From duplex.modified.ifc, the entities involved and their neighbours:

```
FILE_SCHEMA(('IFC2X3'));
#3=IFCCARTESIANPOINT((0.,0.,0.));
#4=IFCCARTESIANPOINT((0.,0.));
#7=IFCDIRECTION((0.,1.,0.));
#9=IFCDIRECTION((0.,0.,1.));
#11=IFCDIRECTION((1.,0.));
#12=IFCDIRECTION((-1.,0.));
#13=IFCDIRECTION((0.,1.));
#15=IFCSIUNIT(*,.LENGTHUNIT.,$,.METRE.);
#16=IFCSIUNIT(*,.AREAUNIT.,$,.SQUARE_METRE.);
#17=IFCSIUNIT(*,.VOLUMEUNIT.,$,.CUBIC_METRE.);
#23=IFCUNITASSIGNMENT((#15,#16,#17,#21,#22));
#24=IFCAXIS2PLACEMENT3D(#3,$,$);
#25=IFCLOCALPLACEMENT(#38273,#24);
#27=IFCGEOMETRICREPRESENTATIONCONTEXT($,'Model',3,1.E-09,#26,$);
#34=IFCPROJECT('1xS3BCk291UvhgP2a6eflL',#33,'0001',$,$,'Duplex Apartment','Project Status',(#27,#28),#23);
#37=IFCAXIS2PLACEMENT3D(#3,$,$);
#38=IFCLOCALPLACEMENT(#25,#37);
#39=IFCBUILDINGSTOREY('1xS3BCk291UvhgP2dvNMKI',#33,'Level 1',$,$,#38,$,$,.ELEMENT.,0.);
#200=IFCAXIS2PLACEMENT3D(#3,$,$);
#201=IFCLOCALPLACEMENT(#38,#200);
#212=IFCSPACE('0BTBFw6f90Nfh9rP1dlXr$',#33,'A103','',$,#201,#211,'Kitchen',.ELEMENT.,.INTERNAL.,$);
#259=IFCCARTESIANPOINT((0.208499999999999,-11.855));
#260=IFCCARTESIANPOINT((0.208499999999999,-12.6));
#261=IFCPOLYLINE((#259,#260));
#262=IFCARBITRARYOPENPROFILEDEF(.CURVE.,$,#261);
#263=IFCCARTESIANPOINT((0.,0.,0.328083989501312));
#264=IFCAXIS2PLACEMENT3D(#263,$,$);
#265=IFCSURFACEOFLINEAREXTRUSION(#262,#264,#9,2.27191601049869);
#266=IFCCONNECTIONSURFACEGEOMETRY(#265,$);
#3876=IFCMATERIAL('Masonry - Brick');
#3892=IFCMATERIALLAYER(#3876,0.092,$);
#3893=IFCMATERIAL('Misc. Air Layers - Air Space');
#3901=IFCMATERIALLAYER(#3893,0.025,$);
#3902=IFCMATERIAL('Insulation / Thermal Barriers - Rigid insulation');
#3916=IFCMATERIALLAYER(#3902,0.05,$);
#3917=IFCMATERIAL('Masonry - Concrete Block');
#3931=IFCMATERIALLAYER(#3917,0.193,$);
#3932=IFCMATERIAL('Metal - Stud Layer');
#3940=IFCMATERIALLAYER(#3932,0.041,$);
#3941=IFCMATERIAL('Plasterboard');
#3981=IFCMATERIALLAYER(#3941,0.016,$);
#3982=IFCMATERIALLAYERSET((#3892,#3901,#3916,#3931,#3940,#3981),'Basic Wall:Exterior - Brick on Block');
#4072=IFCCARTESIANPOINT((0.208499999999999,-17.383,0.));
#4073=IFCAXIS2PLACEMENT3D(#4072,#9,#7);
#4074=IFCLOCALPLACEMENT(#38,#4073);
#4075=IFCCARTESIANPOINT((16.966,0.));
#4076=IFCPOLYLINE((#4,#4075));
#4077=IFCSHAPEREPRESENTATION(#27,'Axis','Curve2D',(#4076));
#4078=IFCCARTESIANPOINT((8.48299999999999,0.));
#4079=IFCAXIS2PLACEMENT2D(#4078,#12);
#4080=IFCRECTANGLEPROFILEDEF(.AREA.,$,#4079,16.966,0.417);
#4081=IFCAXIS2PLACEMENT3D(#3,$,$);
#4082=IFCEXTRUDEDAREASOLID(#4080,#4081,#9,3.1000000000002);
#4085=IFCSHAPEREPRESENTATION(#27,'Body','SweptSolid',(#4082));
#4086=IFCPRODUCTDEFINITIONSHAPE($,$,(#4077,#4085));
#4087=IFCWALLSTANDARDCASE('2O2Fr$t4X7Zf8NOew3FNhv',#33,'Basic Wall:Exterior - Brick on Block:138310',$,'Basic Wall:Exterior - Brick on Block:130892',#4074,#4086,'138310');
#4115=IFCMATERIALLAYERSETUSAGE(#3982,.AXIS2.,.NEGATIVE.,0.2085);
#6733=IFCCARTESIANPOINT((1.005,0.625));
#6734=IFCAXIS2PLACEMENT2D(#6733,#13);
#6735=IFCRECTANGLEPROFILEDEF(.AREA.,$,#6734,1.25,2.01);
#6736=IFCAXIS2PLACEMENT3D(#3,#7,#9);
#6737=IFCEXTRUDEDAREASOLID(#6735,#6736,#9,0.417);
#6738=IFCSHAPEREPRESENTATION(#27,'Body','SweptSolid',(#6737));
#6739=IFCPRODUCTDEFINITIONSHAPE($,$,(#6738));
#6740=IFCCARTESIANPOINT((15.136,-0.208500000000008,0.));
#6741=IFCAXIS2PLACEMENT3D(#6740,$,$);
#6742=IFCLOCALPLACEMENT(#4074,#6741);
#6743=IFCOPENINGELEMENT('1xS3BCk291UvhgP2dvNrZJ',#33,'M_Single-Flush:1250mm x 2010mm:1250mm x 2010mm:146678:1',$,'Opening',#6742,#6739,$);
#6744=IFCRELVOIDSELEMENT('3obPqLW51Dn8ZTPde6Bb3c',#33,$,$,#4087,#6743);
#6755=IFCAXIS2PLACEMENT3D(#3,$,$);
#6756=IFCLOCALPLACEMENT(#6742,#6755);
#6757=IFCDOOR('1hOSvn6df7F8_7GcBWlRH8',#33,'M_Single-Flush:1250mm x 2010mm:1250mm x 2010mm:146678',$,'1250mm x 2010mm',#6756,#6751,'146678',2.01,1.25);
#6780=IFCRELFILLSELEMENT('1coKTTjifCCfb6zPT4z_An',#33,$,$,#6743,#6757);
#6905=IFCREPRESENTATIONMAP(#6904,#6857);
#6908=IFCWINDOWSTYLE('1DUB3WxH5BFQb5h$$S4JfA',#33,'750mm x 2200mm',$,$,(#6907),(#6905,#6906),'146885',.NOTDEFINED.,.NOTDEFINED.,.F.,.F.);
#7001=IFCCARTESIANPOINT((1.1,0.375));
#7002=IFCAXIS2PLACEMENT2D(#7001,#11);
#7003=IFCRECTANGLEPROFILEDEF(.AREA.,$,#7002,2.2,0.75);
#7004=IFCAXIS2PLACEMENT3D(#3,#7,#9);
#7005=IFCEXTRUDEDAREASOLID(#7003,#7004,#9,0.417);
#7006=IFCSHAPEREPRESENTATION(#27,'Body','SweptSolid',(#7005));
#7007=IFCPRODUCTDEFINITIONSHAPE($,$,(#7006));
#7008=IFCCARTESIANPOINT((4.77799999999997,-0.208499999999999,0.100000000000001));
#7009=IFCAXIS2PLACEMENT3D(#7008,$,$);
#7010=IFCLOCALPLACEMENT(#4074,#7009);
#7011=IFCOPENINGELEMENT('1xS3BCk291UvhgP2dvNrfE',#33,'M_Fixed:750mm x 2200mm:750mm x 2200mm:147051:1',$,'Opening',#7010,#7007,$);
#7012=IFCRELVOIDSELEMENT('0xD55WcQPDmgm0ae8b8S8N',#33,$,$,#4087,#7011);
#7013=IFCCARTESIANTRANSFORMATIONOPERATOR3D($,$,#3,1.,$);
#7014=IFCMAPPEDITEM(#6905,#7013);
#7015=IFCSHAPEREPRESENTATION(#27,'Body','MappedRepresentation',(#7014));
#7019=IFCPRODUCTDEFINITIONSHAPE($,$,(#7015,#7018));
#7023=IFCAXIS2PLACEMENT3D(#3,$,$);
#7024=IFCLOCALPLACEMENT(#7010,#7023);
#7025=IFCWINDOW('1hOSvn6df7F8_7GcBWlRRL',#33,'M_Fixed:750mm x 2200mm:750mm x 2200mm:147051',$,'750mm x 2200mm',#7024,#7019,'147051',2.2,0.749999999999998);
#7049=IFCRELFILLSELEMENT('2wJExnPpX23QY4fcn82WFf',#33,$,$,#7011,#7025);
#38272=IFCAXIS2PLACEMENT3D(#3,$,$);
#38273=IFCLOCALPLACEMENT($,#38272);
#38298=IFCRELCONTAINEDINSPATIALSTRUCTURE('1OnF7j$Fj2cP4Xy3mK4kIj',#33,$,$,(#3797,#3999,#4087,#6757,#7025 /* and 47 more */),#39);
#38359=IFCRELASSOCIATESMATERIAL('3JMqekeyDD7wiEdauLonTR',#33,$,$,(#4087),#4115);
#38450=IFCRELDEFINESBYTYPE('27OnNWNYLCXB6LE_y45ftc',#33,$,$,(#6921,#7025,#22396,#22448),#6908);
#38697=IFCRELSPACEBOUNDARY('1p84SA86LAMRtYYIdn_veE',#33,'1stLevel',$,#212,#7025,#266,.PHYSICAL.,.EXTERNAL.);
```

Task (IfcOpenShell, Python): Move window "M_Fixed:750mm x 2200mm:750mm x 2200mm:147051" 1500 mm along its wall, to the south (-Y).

```python
import numpy as np
import ifcopenshell
import ifcopenshell.api.geometry
import ifcopenshell.util.placement

model = ifcopenshell.open("duplex.modified.ifc")

window = model.by_guid("1hOSvn6df7F8_7GcBWlRRL")
opening = window.FillsVoids[0].RelatingOpeningElement
wall = opening.VoidsElements[0].RelatingBuildingElement

wall_matrix = ifcopenshell.util.placement.get_local_placement(wall.ObjectPlacement)
shift = wall_matrix[:3, 0] * -1.5
before = ifcopenshell.util.placement.get_local_placement(window.ObjectPlacement)[:3, 3].copy()

# The window is placed relative to its opening, so it follows when the opening moves.
matrix = ifcopenshell.util.placement.get_local_placement(opening.ObjectPlacement)
matrix[:3, 3] += shift
ifcopenshell.api.geometry.edit_object_placement(
    model, product=opening, matrix=matrix, is_si=False, should_transform_children=True
)

# Space boundary surfaces are stored in each space's coordinates; move them too.
for rel in window.ProvidesBoundaries:
    if not rel.ConnectionGeometry:
        continue
    surface = rel.ConnectionGeometry.SurfaceOnRelatingElement
    space_matrix = ifcopenshell.util.placement.get_local_placement(rel.RelatingSpace.ObjectPlacement)
    point = np.array(surface.Position.Location.Coordinates) + space_matrix[:3, :3].T @ shift
    surface.Position = model.createIfcAxis2Placement3D(
        model.createIfcCartesianPoint(point.tolist()), surface.Position.Axis, surface.Position.RefDirection
    )

after = ifcopenshell.util.placement.get_local_placement(window.ObjectPlacement)[:3, 3]
print("window moved by", (after - before).round(3) + 0.0)

model.write("duplex.modified_updated.ifc")
```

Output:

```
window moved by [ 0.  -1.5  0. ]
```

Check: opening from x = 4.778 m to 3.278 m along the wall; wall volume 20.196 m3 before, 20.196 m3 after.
